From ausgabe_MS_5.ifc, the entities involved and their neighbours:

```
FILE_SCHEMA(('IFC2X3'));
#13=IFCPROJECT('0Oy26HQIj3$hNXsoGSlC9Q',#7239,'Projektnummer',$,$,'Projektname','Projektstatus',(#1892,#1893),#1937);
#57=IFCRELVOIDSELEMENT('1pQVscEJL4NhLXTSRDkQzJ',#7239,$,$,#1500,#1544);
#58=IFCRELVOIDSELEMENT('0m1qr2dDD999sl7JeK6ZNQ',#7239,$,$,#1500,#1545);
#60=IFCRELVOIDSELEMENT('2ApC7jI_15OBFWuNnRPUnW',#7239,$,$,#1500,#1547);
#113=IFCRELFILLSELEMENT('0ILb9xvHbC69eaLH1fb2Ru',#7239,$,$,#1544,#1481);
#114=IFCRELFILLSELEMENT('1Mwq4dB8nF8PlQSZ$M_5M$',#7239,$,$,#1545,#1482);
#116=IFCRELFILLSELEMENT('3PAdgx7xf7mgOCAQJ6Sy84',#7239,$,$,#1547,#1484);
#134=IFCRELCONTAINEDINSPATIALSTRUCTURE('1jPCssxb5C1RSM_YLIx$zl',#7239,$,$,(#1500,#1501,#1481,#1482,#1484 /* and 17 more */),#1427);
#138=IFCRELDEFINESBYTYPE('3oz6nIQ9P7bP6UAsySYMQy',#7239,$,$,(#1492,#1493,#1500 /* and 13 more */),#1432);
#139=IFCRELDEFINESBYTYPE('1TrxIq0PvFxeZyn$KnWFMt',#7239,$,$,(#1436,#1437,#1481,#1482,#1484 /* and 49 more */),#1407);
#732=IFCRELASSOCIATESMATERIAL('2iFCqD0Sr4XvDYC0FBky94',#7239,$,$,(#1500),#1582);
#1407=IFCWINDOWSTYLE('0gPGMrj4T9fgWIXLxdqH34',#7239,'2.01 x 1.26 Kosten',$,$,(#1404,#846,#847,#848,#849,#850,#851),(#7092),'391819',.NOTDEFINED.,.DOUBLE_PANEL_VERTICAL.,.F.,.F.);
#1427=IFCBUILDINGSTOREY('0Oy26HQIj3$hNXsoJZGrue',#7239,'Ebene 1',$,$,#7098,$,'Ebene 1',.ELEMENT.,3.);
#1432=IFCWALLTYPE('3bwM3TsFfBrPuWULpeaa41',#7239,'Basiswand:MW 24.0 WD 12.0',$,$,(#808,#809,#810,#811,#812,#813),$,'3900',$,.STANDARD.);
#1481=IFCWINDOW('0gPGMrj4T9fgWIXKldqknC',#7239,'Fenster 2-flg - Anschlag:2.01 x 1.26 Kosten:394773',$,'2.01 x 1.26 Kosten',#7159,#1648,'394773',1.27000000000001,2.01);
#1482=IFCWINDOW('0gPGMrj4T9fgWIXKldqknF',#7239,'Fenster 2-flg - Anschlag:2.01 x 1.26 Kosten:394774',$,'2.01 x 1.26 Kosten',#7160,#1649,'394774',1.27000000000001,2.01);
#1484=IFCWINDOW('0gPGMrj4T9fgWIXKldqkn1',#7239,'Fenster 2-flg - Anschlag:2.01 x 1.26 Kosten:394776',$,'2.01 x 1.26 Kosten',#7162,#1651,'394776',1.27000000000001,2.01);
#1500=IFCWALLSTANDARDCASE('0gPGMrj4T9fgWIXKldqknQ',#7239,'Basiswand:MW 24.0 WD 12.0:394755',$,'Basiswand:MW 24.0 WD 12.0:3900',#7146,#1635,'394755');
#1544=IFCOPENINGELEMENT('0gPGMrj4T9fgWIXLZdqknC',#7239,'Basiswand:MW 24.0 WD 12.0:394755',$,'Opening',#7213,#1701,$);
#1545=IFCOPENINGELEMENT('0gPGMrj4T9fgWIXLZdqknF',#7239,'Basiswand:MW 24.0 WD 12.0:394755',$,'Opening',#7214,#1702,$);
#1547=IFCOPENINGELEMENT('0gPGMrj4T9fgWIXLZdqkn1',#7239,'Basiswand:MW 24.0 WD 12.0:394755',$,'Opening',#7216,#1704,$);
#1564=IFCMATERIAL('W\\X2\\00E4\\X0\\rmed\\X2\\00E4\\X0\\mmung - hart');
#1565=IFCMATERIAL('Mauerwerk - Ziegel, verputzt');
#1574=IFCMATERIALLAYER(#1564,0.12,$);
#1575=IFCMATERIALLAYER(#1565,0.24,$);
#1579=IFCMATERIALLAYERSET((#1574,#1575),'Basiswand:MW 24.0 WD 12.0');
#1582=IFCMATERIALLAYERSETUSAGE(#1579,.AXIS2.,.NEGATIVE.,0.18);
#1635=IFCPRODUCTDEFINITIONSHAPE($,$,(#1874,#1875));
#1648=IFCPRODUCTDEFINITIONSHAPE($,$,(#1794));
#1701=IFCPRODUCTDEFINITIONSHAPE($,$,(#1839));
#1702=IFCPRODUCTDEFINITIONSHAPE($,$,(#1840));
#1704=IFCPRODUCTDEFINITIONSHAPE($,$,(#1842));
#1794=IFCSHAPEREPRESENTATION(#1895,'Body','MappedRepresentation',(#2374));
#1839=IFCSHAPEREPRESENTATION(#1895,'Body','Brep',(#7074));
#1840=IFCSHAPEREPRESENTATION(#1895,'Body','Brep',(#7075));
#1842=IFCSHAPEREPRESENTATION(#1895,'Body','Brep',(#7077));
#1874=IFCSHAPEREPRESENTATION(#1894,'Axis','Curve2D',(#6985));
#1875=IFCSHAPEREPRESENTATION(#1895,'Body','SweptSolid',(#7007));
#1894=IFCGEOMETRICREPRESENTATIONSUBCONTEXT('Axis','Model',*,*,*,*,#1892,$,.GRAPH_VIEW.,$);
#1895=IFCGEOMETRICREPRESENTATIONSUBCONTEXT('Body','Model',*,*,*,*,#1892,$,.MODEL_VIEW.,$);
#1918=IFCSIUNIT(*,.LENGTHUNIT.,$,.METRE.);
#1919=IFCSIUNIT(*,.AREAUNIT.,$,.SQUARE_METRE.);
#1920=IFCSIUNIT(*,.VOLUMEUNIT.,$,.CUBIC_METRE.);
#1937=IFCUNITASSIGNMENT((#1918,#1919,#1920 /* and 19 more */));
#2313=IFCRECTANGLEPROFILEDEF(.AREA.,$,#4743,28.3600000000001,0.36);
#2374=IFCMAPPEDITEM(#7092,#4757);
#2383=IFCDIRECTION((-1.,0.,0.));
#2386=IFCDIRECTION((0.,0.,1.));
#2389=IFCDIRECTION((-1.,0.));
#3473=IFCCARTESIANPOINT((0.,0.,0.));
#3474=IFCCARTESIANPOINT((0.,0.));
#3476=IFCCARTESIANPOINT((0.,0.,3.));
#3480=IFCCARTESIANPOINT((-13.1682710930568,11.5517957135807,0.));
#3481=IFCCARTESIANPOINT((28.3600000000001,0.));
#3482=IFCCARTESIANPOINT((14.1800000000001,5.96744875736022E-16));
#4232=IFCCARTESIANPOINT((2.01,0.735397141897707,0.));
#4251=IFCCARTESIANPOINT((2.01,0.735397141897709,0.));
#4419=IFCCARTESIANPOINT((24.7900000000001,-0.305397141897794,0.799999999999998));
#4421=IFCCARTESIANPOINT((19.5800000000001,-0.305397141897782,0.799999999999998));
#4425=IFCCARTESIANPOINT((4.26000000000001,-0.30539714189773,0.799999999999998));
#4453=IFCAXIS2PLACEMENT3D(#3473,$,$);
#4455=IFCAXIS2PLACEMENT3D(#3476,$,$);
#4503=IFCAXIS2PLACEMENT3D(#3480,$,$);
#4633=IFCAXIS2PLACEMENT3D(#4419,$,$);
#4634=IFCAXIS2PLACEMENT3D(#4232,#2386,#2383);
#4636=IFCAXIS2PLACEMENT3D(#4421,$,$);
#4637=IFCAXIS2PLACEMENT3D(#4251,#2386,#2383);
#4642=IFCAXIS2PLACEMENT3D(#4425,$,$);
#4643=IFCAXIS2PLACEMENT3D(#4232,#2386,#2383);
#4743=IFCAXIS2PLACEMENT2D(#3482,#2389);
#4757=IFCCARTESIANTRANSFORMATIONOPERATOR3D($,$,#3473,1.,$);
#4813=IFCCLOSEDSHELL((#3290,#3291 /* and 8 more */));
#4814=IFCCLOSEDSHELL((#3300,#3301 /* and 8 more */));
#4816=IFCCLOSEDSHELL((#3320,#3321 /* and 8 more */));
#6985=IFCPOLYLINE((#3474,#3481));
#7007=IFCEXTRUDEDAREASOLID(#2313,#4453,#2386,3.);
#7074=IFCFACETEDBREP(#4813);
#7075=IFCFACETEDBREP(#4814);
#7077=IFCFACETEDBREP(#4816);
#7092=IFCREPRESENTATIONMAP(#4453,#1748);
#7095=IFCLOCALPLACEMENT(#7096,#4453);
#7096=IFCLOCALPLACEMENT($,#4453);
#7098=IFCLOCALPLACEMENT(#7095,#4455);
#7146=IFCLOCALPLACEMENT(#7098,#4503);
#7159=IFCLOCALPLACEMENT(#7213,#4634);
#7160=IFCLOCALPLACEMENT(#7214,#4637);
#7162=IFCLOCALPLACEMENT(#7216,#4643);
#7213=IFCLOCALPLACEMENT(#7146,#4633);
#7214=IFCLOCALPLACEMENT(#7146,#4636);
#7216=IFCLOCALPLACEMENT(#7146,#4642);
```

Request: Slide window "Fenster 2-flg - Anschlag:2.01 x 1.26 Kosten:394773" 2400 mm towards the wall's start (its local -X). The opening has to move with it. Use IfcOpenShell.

```python
import ifcopenshell
import ifcopenshell.api.geometry
import ifcopenshell.util.placement
import ifcopenshell.util.unit

model = ifcopenshell.open("ausgabe_MS_5.ifc")
unit_scale = ifcopenshell.util.unit.calculate_unit_scale(model)

window = model.by_guid("0gPGMrj4T9fgWIXKldqknC")
opening = window.FillsVoids[0].RelatingOpeningElement
wall = opening.VoidsElements[0].RelatingBuildingElement

wall_matrix = ifcopenshell.util.placement.get_local_placement(wall.ObjectPlacement)
shift = wall_matrix[:3, 0] * -2.4 / unit_scale
before = ifcopenshell.util.placement.get_local_placement(window.ObjectPlacement)[:3, 3].copy()

# The window is placed relative to its opening, so it follows when the opening moves.
matrix = ifcopenshell.util.placement.get_local_placement(opening.ObjectPlacement)
matrix[:3, 3] += shift
ifcopenshell.api.geometry.edit_object_placement(
    model, product=opening, matrix=matrix, is_si=False, should_transform_children=True
)

after = ifcopenshell.util.placement.get_local_placement(window.ObjectPlacement)[:3, 3]
print("window moved by", (after - before).round(3) + 0.0)

model.write("ausgabe_MS_5_rev.ifc")
```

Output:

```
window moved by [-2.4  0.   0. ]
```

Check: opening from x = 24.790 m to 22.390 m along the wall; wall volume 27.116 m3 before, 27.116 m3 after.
